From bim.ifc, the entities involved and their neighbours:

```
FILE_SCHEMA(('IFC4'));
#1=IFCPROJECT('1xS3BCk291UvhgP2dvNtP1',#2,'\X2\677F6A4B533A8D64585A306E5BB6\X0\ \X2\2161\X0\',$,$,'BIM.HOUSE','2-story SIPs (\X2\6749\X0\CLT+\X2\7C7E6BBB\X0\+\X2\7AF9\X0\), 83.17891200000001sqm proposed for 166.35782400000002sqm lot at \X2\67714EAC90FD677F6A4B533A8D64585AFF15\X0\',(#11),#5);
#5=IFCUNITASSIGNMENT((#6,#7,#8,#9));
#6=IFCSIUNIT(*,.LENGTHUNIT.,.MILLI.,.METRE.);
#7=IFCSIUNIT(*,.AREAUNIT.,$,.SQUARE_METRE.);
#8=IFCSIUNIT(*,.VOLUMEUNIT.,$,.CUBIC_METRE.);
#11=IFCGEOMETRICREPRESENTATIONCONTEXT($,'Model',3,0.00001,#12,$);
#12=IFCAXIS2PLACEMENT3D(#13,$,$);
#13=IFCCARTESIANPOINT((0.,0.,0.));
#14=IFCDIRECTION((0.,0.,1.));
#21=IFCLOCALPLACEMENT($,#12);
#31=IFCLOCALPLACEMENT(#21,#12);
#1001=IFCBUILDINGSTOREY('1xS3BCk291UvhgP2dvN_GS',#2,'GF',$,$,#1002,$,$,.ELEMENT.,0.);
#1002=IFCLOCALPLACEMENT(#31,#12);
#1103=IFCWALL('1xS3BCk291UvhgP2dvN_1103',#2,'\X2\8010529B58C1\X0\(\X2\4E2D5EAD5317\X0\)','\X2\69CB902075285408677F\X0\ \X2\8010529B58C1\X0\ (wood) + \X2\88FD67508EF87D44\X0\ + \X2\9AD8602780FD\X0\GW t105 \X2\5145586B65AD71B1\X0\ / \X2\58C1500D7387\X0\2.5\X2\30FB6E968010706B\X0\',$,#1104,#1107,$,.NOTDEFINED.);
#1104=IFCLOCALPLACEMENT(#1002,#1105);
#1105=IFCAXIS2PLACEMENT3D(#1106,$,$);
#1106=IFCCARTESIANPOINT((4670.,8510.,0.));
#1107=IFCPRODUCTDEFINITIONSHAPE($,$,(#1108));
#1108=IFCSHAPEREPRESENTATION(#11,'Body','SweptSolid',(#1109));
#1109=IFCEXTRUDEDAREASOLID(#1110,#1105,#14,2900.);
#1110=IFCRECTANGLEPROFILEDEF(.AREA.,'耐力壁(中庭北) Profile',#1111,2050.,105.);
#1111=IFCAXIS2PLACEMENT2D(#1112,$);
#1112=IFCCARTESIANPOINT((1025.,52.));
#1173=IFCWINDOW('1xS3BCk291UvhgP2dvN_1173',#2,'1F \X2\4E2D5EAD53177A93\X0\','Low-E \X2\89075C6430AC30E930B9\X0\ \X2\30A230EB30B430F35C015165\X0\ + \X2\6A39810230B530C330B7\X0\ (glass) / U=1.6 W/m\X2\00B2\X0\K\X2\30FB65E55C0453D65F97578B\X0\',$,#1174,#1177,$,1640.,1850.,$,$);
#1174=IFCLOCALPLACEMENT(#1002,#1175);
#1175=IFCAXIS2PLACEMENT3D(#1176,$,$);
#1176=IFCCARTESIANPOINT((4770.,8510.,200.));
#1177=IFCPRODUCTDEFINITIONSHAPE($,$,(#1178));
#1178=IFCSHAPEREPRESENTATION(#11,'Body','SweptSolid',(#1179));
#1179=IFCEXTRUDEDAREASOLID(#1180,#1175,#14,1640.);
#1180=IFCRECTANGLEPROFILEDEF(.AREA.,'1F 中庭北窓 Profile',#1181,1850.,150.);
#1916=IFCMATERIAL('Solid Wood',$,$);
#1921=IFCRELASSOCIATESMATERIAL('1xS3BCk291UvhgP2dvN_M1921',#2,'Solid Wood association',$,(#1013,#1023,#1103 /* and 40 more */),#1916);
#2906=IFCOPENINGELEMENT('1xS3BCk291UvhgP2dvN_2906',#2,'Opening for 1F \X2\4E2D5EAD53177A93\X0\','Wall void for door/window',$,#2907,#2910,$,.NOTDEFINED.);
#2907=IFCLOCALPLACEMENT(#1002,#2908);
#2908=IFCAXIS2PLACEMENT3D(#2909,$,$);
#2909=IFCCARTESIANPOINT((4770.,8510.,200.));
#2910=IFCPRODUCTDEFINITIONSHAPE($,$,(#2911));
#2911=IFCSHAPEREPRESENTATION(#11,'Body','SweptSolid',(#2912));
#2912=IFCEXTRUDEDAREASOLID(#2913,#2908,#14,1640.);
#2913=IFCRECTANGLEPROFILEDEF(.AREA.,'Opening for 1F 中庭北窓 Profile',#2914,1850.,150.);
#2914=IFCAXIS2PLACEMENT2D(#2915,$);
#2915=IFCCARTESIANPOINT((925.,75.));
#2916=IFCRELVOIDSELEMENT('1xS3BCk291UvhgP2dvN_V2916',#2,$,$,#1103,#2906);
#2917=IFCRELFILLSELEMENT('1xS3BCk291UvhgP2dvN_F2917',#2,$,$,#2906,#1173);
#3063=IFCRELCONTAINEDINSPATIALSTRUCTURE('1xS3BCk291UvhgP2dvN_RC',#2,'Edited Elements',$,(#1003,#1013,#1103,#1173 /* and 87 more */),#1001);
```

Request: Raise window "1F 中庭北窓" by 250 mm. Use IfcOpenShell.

```python
import numpy as np
import ifcopenshell
import ifcopenshell.api.geometry
import ifcopenshell.util.placement
import ifcopenshell.util.unit

model = ifcopenshell.open("bim.ifc")
unit_scale = ifcopenshell.util.unit.calculate_unit_scale(model)

window = model.by_guid("1xS3BCk291UvhgP2dvN_1173")
opening = window.FillsVoids[0].RelatingOpeningElement
dz = 0.25 / unit_scale

shift = np.array([0.0, 0.0, dz])
# The window is not placed relative to its opening, so move both.
for product in (opening, window):
    matrix = ifcopenshell.util.placement.get_local_placement(product.ObjectPlacement)
    matrix[:3, 3] += shift
    ifcopenshell.api.geometry.edit_object_placement(model, product=product, matrix=matrix, is_si=False)

print(f"moved by {dz * unit_scale:+.3f} m")

model.write("bim-out.ifc")
```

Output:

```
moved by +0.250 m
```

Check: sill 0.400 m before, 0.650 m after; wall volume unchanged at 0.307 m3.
